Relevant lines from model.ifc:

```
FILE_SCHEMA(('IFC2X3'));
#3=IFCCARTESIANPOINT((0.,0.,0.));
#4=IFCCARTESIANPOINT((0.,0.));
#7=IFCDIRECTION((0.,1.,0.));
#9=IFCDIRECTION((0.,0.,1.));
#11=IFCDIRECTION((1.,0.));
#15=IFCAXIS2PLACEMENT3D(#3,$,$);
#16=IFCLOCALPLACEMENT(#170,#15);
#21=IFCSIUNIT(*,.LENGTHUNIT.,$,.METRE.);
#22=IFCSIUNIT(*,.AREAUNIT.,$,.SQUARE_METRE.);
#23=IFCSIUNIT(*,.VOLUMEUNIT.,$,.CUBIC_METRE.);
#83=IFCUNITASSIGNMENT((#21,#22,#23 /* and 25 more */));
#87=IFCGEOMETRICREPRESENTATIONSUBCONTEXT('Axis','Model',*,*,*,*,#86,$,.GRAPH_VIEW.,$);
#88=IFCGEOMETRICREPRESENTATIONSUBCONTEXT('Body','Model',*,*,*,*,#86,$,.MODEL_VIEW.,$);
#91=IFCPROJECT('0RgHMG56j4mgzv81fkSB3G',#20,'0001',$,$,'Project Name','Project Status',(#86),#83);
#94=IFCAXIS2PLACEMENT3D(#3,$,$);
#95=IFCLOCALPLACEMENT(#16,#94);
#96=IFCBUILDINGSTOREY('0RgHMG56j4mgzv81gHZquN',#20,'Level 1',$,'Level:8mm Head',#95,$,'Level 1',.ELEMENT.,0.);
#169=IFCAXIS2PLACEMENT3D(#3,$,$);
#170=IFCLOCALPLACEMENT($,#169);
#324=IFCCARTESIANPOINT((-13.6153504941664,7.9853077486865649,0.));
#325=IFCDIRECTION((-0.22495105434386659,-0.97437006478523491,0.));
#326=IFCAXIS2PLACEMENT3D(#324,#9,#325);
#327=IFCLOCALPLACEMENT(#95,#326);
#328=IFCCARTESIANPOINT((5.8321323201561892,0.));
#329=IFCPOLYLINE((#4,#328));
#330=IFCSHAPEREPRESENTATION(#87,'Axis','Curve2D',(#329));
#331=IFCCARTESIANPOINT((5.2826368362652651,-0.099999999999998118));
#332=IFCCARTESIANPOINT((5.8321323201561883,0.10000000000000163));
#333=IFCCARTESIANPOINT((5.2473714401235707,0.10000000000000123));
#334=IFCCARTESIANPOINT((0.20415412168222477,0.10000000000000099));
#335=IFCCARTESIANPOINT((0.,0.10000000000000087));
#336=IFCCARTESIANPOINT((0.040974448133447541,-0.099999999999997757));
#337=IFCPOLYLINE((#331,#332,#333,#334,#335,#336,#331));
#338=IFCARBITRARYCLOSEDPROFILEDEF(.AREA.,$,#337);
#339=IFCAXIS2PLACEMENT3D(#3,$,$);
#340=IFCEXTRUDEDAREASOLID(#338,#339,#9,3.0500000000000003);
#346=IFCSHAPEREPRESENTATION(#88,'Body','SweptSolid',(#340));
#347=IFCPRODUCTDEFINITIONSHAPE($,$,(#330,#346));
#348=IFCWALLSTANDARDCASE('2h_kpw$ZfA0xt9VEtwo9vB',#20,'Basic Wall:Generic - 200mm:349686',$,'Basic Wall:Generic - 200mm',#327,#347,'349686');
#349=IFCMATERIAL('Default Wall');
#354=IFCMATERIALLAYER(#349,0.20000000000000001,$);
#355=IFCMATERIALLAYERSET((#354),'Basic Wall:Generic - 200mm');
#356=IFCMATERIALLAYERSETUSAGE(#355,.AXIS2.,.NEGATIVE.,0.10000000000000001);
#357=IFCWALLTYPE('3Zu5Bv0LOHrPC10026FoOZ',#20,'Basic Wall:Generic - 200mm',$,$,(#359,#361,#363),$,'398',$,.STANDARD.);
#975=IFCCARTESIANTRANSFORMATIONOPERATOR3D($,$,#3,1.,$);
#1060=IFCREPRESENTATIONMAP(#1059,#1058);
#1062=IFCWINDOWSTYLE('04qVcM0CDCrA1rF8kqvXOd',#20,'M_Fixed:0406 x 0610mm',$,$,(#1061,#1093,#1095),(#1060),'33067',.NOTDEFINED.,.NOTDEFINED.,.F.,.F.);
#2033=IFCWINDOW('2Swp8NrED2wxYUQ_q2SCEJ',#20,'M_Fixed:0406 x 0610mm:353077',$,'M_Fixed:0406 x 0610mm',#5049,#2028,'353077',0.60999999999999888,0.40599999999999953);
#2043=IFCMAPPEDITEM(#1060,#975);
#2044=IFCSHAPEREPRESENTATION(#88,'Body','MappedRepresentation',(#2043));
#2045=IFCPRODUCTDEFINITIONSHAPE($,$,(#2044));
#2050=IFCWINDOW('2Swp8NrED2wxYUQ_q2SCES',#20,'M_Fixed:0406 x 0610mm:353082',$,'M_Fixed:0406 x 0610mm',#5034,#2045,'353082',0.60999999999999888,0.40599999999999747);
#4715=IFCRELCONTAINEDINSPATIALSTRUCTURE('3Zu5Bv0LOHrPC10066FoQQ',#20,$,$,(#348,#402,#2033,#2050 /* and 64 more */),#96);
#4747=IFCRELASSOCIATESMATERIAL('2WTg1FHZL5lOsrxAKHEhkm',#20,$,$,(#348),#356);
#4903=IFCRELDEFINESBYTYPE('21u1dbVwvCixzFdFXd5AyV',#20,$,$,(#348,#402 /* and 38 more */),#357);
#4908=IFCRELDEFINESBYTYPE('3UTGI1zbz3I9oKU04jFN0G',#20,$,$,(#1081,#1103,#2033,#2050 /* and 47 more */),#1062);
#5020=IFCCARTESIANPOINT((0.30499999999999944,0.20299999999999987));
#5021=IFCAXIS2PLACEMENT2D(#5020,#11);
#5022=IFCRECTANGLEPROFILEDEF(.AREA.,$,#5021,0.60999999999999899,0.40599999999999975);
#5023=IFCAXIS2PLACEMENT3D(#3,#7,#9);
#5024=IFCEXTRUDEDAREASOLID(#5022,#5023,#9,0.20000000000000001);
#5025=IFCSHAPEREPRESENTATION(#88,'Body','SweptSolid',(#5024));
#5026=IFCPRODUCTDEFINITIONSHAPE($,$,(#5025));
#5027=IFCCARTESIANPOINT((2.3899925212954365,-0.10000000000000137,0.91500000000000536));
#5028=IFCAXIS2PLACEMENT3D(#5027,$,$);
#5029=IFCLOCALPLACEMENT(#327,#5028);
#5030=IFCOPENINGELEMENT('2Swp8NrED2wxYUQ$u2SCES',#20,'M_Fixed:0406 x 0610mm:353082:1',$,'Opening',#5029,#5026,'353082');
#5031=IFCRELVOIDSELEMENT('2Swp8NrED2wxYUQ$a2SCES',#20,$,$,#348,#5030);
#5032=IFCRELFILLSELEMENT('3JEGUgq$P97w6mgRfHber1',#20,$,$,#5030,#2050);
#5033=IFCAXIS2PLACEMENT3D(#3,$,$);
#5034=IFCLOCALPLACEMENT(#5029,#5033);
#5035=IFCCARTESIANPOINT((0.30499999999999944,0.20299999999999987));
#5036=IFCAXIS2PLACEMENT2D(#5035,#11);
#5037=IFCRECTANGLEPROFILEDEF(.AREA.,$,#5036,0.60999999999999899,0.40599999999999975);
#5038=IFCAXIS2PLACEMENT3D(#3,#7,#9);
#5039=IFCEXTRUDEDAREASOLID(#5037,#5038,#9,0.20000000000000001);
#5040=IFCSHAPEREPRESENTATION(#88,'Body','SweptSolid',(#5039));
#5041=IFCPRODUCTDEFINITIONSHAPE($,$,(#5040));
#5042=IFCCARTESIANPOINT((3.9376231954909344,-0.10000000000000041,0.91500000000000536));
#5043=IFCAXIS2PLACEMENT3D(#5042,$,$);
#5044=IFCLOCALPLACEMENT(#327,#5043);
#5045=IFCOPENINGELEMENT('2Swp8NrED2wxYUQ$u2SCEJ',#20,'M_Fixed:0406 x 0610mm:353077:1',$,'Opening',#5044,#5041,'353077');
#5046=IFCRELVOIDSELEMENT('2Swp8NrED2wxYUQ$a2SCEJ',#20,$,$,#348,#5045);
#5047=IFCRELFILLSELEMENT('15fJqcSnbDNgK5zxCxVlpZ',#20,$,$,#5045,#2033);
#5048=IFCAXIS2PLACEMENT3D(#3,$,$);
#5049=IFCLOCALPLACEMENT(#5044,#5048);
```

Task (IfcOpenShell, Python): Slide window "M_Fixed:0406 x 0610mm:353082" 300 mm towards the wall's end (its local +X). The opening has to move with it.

```python
import ifcopenshell
import ifcopenshell.api.geometry
import ifcopenshell.util.placement

model = ifcopenshell.open("model.ifc")

window = model.by_id(2050)
opening = window.FillsVoids[0].RelatingOpeningElement
wall = opening.VoidsElements[0].RelatingBuildingElement

wall_matrix = ifcopenshell.util.placement.get_local_placement(wall.ObjectPlacement)
shift = wall_matrix[:3, 0] * 0.3
before = ifcopenshell.util.placement.get_local_placement(window.ObjectPlacement)[:3, 3].copy()

# The window is placed relative to its opening, so it follows when the opening moves.
matrix = ifcopenshell.util.placement.get_local_placement(opening.ObjectPlacement)
matrix[:3, 3] += shift
ifcopenshell.api.geometry.edit_object_placement(
    model, product=opening, matrix=matrix, is_si=False, should_transform_children=True
)

after = ifcopenshell.util.placement.get_local_placement(window.ObjectPlacement)[:3, 3]
print("window moved by", (after - before).round(3) + 0.0)

model.write("model_rev.ifc")
```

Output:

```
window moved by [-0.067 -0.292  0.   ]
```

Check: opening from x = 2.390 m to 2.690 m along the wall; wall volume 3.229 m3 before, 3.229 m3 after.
